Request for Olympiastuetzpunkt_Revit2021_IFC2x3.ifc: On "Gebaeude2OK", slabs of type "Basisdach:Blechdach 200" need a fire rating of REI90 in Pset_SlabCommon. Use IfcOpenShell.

First a look at what the model holds.

```python
import ifcopenshell
import ifcopenshell.util.element

model = ifcopenshell.open("Olympiastuetzpunkt_Revit2021_IFC2x3.ifc")
print(model.schema)
storey = next(s for s in model.by_type("IfcBuildingStorey") if s.Name == "Gebaeude2OK")
slabs = [e for e in ifcopenshell.util.element.get_decomposition(storey) if e.is_a("IfcSlab")]
seen = {}
for e in slabs:
    element_type = ifcopenshell.util.element.get_type(e)
    key = (element_type.Name if element_type != e and element_type else None, ifcopenshell.util.element.get_pset(e, "Pset_SlabCommon", "FireRating"))
    seen[key] = seen.get(key, 0) + 1
for (name, value), count in sorted(seen.items(), key=str):
    print(count, "x", name, "|", value)
```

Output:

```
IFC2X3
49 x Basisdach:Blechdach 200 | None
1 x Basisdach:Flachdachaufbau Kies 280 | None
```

```python
import ifcopenshell
import ifcopenshell.api.pset
import ifcopenshell.util.element

model = ifcopenshell.open("Olympiastuetzpunkt_Revit2021_IFC2x3.ifc")

storey = next(s for s in model.by_type("IfcBuildingStorey") if s.Name == "Gebaeude2OK")
slabs = [e for e in ifcopenshell.util.element.get_decomposition(storey) if e.is_a("IfcSlab")]

count = 0
for e in slabs:
    element_type = ifcopenshell.util.element.get_type(e)
    if element_type in (None, e) or element_type.Name != "Basisdach:Blechdach 200":
        continue
    # add_pset returns the element's existing set when there is one.
    pset = ifcopenshell.api.pset.add_pset(model, product=e, name="Pset_SlabCommon")
    ifcopenshell.api.pset.edit_pset(model, pset=pset, properties={"FireRating": "REI90"})
    count += 1

print(count, "slabs updated")

model.write("Olympiastuetzpunkt_Revit2021_IFC2x3_rev.ifc")
```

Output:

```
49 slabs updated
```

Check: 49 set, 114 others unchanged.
